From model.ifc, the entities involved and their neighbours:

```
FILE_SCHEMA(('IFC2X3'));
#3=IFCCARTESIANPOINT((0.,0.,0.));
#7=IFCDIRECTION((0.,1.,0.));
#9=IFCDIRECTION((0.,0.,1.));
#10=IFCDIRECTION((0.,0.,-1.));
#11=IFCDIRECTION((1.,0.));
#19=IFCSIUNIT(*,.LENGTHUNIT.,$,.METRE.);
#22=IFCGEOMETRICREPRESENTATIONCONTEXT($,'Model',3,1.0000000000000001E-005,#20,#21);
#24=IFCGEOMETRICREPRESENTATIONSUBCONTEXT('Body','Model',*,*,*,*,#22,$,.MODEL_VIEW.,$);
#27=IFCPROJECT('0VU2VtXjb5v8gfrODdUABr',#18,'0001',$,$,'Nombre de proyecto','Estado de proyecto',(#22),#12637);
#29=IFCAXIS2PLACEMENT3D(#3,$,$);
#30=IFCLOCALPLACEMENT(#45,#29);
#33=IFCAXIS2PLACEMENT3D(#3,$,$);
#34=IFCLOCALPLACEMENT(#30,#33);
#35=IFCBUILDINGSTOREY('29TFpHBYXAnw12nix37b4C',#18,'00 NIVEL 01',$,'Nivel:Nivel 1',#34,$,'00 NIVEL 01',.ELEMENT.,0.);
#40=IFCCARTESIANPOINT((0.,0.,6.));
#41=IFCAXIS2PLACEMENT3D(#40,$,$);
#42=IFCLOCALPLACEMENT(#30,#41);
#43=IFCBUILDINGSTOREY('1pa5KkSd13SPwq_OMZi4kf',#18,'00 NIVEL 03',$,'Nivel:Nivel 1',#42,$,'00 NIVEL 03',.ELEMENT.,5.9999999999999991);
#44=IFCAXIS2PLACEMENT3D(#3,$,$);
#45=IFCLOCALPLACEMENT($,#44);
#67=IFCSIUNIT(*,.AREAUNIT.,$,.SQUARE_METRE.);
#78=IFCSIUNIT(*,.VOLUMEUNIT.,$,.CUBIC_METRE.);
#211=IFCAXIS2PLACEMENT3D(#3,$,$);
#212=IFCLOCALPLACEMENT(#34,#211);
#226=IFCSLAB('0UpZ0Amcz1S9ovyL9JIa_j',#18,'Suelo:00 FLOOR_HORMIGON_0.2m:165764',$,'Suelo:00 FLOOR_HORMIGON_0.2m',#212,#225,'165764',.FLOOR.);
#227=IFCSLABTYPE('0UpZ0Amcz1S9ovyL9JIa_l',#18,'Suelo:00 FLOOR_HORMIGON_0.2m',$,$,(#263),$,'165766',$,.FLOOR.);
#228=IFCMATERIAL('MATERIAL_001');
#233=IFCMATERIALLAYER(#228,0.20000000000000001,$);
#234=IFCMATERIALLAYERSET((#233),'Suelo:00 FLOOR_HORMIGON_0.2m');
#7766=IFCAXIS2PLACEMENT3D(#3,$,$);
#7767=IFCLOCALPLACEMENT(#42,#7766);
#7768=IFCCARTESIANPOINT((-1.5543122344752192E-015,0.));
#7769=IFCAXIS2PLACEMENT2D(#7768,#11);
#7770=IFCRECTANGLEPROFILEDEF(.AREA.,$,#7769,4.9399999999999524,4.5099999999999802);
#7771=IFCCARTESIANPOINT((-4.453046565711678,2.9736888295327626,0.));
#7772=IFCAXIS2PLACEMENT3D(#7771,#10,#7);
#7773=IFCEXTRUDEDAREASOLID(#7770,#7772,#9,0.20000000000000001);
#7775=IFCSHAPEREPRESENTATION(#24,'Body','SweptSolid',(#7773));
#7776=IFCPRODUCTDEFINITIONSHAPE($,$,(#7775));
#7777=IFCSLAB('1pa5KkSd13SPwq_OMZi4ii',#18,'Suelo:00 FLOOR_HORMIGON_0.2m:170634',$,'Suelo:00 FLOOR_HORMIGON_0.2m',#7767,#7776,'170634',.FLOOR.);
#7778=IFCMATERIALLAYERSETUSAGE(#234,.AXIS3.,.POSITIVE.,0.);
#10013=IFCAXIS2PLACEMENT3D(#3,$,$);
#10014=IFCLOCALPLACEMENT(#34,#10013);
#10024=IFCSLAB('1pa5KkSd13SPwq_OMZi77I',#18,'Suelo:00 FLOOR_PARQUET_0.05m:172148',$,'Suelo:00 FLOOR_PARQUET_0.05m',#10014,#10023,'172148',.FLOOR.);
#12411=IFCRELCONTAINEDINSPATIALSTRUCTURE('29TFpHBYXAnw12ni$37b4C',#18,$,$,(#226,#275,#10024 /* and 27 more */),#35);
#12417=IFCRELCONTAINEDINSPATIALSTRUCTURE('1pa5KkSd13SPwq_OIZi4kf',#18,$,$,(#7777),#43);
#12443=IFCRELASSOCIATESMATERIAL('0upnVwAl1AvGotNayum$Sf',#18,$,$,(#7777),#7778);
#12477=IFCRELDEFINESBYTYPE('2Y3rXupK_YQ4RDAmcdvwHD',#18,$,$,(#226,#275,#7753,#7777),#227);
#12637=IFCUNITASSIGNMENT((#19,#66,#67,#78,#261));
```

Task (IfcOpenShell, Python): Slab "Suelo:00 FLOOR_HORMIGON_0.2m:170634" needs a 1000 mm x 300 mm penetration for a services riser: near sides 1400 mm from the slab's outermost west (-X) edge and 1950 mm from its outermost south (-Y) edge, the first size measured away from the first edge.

```python
import numpy as np
import ifcopenshell
import ifcopenshell.api.feature
import ifcopenshell.api.geometry
import ifcopenshell.api.root
import ifcopenshell.geom
import ifcopenshell.util.placement
import ifcopenshell.util.representation
import ifcopenshell.util.shape
import ifcopenshell.util.unit

model = ifcopenshell.open("model.ifc")
unit_scale = ifcopenshell.util.unit.calculate_unit_scale(model)
settings = ifcopenshell.geom.settings()


def volume(element):
    """Net volume in cubic metres, openings subtracted."""
    shape = ifcopenshell.geom.create_shape(settings, element)
    return ifcopenshell.util.shape.get_volume(shape.geometry)


slab = model.by_guid("1pa5KkSd13SPwq_OMZi4ii")
before = volume(slab)

# Extent in the slab's own axes, in metres. The edges named are its -X and -Y sides.
slab_shape = ifcopenshell.geom.create_shape(settings, slab)
vertices = ifcopenshell.util.shape.get_vertices(slab_shape.geometry)
x_min, y_min, bottom = vertices.min(axis=0)
top = vertices[:, 2].max()

opening = ifcopenshell.api.root.create_entity(model, ifc_class="IfcOpeningElement", name="Services riser opening")
context = ifcopenshell.util.representation.get_context(model, "Model", "Body", "MODEL_VIEW")
width, depth = 1, 0.3
outline = [(0.0, 0.0), (width, 0.0), (width, depth), (0.0, depth), (0.0, 0.0)]
# Overshoot both faces by 50 mm so the cut is clean.
shape = ifcopenshell.api.geometry.add_slab_representation(
    model, context=context, depth=top - bottom + 0.1, polyline=outline
)
ifcopenshell.api.geometry.assign_representation(model, product=opening, representation=shape)

matrix = ifcopenshell.util.placement.get_local_placement(slab.ObjectPlacement)
matrix[:, 3] = matrix @ np.append(np.array([x_min + 1.4, y_min + 1.95, bottom - 0.05]) / unit_scale, 1.0)
ifcopenshell.api.geometry.edit_object_placement(model, product=opening, matrix=matrix, is_si=False)
ifcopenshell.api.feature.add_feature(model, feature=opening, element=slab)

after = volume(slab)

print(f"slab volume {before:.3f} -> {after:.3f} m3")

model.write("model_rev.ifc")
```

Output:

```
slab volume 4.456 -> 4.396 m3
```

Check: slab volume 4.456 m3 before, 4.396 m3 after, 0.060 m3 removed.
